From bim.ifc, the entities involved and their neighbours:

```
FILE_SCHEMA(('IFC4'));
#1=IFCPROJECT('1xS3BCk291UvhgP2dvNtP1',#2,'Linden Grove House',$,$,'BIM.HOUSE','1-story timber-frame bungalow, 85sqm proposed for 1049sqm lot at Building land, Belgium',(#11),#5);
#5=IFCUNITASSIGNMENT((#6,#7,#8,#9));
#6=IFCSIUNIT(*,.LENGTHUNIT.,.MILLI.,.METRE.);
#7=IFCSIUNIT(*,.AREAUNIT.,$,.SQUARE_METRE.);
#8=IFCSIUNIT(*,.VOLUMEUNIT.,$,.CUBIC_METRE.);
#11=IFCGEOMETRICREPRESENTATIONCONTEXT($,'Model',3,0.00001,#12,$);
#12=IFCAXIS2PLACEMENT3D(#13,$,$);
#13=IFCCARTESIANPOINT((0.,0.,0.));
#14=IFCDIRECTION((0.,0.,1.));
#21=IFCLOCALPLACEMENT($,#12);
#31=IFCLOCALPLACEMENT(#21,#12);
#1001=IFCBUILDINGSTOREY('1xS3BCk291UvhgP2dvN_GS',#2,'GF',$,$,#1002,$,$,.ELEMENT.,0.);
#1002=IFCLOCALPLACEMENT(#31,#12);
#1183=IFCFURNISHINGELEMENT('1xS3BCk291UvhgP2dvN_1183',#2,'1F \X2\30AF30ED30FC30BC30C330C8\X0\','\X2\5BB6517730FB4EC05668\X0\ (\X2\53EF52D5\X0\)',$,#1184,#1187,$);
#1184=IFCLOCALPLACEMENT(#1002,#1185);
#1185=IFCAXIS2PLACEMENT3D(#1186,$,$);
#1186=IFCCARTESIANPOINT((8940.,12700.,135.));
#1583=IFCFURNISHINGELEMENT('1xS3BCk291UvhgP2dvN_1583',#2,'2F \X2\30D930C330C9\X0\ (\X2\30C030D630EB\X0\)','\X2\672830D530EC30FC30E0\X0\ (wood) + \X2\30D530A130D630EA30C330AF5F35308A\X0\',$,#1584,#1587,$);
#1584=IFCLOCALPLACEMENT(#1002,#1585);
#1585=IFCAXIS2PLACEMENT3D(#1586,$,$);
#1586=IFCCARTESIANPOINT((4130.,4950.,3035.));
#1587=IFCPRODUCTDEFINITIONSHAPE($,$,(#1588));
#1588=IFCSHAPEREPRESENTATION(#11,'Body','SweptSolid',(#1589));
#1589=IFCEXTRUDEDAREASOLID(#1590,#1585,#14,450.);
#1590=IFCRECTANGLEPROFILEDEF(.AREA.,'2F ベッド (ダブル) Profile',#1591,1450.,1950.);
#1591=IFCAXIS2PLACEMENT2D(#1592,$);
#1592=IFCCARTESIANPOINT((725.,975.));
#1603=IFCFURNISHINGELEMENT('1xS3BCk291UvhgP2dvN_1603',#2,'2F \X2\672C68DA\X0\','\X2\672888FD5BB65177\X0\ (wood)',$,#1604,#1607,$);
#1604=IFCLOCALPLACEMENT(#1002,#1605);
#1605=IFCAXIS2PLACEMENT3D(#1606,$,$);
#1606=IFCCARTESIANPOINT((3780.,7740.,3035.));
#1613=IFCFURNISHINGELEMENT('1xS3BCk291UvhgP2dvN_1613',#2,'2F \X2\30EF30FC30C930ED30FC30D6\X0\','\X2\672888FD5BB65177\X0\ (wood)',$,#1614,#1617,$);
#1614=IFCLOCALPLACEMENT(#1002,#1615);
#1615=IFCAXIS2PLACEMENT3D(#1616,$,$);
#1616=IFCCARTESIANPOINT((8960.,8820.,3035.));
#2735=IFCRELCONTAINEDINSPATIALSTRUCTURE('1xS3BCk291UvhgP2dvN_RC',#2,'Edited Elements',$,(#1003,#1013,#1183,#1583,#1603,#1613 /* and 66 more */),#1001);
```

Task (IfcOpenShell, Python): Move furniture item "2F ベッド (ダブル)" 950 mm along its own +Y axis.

```python
import ifcopenshell
import ifcopenshell.api.geometry
import ifcopenshell.util.placement
import ifcopenshell.util.unit

model = ifcopenshell.open("bim.ifc")
unit_scale = ifcopenshell.util.unit.calculate_unit_scale(model)

item = model.by_guid("1xS3BCk291UvhgP2dvN_1583")
matrix = ifcopenshell.util.placement.get_local_placement(item.ObjectPlacement)
matrix[:3, 3] += matrix[:3, 1] * 0.95 / unit_scale
ifcopenshell.api.geometry.edit_object_placement(model, product=item, matrix=matrix, is_si=False)

print(ifcopenshell.util.placement.get_local_placement(item.ObjectPlacement).round(3) + 0.0)

model.write("bim_v2.ifc")
```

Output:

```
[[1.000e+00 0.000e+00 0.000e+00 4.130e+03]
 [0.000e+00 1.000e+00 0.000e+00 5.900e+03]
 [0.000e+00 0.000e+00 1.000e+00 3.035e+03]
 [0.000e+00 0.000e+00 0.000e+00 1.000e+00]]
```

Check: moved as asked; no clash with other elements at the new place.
